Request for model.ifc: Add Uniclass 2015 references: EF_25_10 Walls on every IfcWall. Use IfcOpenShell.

First a look at what the model holds.

```python
import ifcopenshell

model = ifcopenshell.open("model.ifc")
print(model.schema)
print("classifications:", [c.Name for c in model.by_type("IfcClassification")])
for ifc_class in ("IfcDoor", "IfcRoof", "IfcStair", "IfcWall", "IfcWindow"):
    print(ifc_class, len(model.by_type(ifc_class)))
```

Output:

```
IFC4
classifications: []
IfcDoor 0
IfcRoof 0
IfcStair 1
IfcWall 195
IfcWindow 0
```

```python
import ifcopenshell
import ifcopenshell.api.classification

model = ifcopenshell.open("model.ifc")

system = ifcopenshell.api.classification.add_classification(model, classification="Uniclass 2015")

codes = {
    "IfcWall": ("EF_25_10", "Walls"),
}
for ifc_class, (code, name) in codes.items():
    products = model.by_type(ifc_class)
    ifcopenshell.api.classification.add_reference(
        model, products=products, classification=system, identification=code, name=name
    )
    print(code, len(products))

model.write("model_rev.ifc")
```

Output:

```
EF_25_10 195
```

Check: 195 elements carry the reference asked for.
